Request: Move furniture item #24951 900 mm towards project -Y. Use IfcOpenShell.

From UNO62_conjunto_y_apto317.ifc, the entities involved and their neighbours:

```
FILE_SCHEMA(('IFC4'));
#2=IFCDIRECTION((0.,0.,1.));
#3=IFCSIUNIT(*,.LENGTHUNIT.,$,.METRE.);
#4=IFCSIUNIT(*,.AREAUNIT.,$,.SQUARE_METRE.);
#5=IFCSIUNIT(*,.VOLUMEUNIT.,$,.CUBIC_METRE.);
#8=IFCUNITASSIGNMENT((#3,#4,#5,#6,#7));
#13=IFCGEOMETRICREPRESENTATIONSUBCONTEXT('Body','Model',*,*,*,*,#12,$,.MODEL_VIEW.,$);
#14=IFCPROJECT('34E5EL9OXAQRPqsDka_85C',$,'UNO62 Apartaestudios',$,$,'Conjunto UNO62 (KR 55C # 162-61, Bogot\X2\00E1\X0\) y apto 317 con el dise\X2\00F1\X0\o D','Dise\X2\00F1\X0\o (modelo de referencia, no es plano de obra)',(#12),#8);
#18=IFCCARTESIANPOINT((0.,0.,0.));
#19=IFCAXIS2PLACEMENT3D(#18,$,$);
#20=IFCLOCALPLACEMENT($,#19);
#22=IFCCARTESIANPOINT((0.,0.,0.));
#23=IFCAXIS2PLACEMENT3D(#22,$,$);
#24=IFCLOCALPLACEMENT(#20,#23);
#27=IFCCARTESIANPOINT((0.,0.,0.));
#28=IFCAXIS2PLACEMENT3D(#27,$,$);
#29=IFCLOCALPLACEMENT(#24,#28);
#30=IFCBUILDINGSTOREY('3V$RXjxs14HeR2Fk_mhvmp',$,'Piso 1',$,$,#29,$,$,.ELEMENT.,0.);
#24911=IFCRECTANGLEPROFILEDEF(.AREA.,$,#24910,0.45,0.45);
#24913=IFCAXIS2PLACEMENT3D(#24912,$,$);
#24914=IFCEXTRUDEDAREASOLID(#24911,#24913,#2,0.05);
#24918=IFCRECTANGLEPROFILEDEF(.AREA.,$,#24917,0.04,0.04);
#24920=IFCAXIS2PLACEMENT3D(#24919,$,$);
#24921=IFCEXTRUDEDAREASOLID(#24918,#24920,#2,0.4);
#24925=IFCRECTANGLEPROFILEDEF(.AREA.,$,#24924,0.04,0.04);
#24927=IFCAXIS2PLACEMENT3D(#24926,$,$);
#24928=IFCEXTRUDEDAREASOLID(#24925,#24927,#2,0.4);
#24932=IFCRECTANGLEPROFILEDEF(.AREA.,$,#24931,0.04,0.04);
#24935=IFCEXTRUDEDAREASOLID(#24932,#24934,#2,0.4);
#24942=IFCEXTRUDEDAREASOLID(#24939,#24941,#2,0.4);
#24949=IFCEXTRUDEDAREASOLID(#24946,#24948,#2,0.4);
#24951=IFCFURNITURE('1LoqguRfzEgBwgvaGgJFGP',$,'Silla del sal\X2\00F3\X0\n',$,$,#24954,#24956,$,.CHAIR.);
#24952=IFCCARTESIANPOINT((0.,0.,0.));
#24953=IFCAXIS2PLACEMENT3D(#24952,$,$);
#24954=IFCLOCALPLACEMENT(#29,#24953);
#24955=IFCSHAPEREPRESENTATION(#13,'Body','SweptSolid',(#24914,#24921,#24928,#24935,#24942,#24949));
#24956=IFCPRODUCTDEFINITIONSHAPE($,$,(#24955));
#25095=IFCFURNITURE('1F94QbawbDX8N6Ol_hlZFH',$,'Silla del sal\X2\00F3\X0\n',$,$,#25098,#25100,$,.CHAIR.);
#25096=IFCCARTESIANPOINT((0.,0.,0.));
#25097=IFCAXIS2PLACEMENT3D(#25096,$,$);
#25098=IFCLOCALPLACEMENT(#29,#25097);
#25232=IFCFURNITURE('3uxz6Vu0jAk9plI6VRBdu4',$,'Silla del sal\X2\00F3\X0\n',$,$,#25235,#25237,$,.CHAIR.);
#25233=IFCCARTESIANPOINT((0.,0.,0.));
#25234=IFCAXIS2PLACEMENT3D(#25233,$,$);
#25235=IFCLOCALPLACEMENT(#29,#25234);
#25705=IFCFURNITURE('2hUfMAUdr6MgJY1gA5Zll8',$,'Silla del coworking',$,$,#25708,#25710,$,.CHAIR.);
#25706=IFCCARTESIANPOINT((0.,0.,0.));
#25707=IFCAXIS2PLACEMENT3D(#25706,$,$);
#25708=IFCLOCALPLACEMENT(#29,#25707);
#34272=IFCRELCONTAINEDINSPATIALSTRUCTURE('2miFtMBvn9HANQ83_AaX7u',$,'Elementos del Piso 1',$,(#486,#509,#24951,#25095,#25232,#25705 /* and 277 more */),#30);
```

```python
import ifcopenshell
import ifcopenshell.api.geometry
import ifcopenshell.util.placement
import ifcopenshell.util.unit

model = ifcopenshell.open("UNO62_conjunto_y_apto317.ifc")
unit_scale = ifcopenshell.util.unit.calculate_unit_scale(model)

item = model.by_guid("1LoqguRfzEgBwgvaGgJFGP")
matrix = ifcopenshell.util.placement.get_local_placement(item.ObjectPlacement)
matrix[1, 3] -= 0.9 / unit_scale
ifcopenshell.api.geometry.edit_object_placement(model, product=item, matrix=matrix, is_si=False)

print(ifcopenshell.util.placement.get_local_placement(item.ObjectPlacement).round(3) + 0.0)

model.write("UNO62_conjunto_y_apto317-out.ifc")
```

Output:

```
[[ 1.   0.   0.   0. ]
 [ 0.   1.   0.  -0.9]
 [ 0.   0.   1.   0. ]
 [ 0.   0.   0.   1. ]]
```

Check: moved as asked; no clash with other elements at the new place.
